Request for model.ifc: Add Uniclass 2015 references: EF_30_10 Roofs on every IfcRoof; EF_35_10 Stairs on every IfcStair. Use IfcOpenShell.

First a look at what the model holds.

```python
import ifcopenshell

model = ifcopenshell.open("model.ifc")
print(model.schema)
print("classifications:", [c.Name for c in model.by_type("IfcClassification")])
for ifc_class in ("IfcDoor", "IfcRoof", "IfcStair", "IfcWall", "IfcWindow"):
    print(ifc_class, len(model.by_type(ifc_class)))
```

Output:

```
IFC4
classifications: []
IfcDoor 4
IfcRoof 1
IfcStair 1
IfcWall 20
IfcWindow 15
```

```python
import ifcopenshell
import ifcopenshell.api.classification

model = ifcopenshell.open("model.ifc")

system = ifcopenshell.api.classification.add_classification(model, classification="Uniclass 2015")

codes = {
    "IfcRoof": ("EF_30_10", "Roofs"),
    "IfcStair": ("EF_35_10", "Stairs"),
}
for ifc_class, (code, name) in codes.items():
    products = model.by_type(ifc_class)
    ifcopenshell.api.classification.add_reference(
        model, products=products, classification=system, identification=code, name=name
    )
    print(code, len(products))

model.write("model_v2.ifc")
```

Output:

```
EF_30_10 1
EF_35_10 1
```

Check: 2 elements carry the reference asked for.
